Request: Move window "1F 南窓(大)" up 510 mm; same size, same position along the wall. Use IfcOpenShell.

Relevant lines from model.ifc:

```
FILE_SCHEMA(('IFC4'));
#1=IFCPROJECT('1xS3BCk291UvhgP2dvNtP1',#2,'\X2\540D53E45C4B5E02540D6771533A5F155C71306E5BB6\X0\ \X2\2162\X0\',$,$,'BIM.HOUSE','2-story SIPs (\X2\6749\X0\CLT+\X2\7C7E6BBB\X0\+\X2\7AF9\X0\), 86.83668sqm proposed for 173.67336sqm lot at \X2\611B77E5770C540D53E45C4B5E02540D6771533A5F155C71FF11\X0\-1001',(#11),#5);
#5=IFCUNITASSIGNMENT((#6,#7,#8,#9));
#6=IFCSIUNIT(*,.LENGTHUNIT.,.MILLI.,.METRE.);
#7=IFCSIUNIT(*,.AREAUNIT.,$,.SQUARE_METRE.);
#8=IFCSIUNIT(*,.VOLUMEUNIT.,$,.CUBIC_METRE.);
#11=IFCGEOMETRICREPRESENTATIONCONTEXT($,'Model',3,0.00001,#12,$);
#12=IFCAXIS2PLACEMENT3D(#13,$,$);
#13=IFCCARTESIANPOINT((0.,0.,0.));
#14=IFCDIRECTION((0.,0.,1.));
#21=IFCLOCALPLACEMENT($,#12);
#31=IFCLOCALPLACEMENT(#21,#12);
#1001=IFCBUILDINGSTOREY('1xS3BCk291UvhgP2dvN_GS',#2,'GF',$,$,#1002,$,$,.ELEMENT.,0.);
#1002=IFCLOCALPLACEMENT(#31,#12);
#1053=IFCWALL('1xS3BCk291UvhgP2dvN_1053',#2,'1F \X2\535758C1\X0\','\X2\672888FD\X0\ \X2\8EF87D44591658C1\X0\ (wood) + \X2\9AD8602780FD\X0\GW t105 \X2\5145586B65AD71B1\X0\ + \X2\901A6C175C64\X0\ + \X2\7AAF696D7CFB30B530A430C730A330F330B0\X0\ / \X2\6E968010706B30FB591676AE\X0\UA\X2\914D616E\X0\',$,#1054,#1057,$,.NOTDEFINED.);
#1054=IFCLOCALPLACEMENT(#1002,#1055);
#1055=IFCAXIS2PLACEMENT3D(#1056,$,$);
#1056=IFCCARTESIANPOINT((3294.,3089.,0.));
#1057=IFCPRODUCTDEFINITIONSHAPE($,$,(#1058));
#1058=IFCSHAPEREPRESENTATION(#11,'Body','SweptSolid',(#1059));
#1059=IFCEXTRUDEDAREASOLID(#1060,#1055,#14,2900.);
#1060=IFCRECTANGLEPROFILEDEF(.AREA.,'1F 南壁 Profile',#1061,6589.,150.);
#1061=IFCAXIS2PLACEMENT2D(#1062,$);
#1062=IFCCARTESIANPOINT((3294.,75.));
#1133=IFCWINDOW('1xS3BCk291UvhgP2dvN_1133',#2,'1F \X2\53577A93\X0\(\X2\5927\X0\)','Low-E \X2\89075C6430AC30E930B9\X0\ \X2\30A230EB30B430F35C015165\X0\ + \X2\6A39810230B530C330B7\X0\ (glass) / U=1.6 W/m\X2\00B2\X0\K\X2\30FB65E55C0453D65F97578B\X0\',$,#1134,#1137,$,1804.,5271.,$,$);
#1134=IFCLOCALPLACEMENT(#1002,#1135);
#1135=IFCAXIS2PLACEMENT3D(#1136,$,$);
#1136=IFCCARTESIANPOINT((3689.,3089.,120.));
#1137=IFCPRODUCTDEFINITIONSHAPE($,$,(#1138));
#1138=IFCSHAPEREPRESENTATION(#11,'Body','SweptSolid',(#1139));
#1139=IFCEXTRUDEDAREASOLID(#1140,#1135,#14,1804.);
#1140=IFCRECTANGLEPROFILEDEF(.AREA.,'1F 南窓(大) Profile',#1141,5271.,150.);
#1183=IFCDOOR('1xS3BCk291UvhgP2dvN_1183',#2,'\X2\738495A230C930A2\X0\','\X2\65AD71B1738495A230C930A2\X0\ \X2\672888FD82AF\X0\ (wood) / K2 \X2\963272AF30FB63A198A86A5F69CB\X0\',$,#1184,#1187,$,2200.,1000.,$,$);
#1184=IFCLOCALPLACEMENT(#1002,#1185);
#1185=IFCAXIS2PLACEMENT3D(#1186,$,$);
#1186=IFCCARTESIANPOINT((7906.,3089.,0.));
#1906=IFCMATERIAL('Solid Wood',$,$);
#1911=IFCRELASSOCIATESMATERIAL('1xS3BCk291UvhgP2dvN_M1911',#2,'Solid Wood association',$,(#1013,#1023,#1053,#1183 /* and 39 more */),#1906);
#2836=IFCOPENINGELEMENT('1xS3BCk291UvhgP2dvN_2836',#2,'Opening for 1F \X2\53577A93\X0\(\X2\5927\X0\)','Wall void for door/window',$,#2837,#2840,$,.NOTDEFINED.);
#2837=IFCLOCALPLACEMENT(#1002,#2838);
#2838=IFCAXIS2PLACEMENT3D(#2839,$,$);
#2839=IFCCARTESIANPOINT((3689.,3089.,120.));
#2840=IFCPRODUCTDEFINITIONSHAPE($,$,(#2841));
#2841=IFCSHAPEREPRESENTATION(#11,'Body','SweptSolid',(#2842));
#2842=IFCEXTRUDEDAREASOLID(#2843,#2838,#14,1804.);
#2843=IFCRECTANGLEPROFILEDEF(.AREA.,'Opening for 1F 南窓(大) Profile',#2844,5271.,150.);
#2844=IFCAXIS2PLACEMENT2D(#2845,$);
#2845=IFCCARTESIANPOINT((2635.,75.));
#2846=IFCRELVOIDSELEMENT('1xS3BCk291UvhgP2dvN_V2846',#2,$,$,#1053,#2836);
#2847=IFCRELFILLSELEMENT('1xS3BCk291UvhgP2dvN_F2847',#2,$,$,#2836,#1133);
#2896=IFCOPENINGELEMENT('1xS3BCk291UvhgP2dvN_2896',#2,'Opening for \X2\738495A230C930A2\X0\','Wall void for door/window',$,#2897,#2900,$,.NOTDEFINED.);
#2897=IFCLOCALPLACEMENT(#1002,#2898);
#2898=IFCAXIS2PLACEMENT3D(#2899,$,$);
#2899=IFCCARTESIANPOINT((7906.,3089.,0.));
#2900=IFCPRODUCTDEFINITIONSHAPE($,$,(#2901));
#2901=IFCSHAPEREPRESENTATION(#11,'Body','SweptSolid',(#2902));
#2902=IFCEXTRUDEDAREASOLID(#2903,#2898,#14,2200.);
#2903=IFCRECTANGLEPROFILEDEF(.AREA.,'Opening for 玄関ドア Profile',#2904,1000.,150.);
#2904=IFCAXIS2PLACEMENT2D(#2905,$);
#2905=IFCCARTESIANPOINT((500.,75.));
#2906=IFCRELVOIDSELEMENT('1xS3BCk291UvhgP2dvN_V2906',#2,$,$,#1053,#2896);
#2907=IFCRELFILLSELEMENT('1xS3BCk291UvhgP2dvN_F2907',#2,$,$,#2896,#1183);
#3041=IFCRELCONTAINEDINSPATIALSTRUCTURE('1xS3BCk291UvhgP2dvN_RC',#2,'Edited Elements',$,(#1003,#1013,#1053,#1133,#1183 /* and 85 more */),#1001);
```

```python
import numpy as np
import ifcopenshell
import ifcopenshell.api.geometry
import ifcopenshell.util.placement
import ifcopenshell.util.unit

model = ifcopenshell.open("model.ifc")
unit_scale = ifcopenshell.util.unit.calculate_unit_scale(model)

window = model.by_guid("1xS3BCk291UvhgP2dvN_1133")
opening = window.FillsVoids[0].RelatingOpeningElement
dz = 0.51 / unit_scale

shift = np.array([0.0, 0.0, dz])
# The window is not placed relative to its opening, so move both.
for product in (opening, window):
    matrix = ifcopenshell.util.placement.get_local_placement(product.ObjectPlacement)
    matrix[:3, 3] += shift
    ifcopenshell.api.geometry.edit_object_placement(model, product=product, matrix=matrix, is_si=False)

print(f"moved by {dz * unit_scale:+.3f} m")

model.write("model_updated.ifc")
```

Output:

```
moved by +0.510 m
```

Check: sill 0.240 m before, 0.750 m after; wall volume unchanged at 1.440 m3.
